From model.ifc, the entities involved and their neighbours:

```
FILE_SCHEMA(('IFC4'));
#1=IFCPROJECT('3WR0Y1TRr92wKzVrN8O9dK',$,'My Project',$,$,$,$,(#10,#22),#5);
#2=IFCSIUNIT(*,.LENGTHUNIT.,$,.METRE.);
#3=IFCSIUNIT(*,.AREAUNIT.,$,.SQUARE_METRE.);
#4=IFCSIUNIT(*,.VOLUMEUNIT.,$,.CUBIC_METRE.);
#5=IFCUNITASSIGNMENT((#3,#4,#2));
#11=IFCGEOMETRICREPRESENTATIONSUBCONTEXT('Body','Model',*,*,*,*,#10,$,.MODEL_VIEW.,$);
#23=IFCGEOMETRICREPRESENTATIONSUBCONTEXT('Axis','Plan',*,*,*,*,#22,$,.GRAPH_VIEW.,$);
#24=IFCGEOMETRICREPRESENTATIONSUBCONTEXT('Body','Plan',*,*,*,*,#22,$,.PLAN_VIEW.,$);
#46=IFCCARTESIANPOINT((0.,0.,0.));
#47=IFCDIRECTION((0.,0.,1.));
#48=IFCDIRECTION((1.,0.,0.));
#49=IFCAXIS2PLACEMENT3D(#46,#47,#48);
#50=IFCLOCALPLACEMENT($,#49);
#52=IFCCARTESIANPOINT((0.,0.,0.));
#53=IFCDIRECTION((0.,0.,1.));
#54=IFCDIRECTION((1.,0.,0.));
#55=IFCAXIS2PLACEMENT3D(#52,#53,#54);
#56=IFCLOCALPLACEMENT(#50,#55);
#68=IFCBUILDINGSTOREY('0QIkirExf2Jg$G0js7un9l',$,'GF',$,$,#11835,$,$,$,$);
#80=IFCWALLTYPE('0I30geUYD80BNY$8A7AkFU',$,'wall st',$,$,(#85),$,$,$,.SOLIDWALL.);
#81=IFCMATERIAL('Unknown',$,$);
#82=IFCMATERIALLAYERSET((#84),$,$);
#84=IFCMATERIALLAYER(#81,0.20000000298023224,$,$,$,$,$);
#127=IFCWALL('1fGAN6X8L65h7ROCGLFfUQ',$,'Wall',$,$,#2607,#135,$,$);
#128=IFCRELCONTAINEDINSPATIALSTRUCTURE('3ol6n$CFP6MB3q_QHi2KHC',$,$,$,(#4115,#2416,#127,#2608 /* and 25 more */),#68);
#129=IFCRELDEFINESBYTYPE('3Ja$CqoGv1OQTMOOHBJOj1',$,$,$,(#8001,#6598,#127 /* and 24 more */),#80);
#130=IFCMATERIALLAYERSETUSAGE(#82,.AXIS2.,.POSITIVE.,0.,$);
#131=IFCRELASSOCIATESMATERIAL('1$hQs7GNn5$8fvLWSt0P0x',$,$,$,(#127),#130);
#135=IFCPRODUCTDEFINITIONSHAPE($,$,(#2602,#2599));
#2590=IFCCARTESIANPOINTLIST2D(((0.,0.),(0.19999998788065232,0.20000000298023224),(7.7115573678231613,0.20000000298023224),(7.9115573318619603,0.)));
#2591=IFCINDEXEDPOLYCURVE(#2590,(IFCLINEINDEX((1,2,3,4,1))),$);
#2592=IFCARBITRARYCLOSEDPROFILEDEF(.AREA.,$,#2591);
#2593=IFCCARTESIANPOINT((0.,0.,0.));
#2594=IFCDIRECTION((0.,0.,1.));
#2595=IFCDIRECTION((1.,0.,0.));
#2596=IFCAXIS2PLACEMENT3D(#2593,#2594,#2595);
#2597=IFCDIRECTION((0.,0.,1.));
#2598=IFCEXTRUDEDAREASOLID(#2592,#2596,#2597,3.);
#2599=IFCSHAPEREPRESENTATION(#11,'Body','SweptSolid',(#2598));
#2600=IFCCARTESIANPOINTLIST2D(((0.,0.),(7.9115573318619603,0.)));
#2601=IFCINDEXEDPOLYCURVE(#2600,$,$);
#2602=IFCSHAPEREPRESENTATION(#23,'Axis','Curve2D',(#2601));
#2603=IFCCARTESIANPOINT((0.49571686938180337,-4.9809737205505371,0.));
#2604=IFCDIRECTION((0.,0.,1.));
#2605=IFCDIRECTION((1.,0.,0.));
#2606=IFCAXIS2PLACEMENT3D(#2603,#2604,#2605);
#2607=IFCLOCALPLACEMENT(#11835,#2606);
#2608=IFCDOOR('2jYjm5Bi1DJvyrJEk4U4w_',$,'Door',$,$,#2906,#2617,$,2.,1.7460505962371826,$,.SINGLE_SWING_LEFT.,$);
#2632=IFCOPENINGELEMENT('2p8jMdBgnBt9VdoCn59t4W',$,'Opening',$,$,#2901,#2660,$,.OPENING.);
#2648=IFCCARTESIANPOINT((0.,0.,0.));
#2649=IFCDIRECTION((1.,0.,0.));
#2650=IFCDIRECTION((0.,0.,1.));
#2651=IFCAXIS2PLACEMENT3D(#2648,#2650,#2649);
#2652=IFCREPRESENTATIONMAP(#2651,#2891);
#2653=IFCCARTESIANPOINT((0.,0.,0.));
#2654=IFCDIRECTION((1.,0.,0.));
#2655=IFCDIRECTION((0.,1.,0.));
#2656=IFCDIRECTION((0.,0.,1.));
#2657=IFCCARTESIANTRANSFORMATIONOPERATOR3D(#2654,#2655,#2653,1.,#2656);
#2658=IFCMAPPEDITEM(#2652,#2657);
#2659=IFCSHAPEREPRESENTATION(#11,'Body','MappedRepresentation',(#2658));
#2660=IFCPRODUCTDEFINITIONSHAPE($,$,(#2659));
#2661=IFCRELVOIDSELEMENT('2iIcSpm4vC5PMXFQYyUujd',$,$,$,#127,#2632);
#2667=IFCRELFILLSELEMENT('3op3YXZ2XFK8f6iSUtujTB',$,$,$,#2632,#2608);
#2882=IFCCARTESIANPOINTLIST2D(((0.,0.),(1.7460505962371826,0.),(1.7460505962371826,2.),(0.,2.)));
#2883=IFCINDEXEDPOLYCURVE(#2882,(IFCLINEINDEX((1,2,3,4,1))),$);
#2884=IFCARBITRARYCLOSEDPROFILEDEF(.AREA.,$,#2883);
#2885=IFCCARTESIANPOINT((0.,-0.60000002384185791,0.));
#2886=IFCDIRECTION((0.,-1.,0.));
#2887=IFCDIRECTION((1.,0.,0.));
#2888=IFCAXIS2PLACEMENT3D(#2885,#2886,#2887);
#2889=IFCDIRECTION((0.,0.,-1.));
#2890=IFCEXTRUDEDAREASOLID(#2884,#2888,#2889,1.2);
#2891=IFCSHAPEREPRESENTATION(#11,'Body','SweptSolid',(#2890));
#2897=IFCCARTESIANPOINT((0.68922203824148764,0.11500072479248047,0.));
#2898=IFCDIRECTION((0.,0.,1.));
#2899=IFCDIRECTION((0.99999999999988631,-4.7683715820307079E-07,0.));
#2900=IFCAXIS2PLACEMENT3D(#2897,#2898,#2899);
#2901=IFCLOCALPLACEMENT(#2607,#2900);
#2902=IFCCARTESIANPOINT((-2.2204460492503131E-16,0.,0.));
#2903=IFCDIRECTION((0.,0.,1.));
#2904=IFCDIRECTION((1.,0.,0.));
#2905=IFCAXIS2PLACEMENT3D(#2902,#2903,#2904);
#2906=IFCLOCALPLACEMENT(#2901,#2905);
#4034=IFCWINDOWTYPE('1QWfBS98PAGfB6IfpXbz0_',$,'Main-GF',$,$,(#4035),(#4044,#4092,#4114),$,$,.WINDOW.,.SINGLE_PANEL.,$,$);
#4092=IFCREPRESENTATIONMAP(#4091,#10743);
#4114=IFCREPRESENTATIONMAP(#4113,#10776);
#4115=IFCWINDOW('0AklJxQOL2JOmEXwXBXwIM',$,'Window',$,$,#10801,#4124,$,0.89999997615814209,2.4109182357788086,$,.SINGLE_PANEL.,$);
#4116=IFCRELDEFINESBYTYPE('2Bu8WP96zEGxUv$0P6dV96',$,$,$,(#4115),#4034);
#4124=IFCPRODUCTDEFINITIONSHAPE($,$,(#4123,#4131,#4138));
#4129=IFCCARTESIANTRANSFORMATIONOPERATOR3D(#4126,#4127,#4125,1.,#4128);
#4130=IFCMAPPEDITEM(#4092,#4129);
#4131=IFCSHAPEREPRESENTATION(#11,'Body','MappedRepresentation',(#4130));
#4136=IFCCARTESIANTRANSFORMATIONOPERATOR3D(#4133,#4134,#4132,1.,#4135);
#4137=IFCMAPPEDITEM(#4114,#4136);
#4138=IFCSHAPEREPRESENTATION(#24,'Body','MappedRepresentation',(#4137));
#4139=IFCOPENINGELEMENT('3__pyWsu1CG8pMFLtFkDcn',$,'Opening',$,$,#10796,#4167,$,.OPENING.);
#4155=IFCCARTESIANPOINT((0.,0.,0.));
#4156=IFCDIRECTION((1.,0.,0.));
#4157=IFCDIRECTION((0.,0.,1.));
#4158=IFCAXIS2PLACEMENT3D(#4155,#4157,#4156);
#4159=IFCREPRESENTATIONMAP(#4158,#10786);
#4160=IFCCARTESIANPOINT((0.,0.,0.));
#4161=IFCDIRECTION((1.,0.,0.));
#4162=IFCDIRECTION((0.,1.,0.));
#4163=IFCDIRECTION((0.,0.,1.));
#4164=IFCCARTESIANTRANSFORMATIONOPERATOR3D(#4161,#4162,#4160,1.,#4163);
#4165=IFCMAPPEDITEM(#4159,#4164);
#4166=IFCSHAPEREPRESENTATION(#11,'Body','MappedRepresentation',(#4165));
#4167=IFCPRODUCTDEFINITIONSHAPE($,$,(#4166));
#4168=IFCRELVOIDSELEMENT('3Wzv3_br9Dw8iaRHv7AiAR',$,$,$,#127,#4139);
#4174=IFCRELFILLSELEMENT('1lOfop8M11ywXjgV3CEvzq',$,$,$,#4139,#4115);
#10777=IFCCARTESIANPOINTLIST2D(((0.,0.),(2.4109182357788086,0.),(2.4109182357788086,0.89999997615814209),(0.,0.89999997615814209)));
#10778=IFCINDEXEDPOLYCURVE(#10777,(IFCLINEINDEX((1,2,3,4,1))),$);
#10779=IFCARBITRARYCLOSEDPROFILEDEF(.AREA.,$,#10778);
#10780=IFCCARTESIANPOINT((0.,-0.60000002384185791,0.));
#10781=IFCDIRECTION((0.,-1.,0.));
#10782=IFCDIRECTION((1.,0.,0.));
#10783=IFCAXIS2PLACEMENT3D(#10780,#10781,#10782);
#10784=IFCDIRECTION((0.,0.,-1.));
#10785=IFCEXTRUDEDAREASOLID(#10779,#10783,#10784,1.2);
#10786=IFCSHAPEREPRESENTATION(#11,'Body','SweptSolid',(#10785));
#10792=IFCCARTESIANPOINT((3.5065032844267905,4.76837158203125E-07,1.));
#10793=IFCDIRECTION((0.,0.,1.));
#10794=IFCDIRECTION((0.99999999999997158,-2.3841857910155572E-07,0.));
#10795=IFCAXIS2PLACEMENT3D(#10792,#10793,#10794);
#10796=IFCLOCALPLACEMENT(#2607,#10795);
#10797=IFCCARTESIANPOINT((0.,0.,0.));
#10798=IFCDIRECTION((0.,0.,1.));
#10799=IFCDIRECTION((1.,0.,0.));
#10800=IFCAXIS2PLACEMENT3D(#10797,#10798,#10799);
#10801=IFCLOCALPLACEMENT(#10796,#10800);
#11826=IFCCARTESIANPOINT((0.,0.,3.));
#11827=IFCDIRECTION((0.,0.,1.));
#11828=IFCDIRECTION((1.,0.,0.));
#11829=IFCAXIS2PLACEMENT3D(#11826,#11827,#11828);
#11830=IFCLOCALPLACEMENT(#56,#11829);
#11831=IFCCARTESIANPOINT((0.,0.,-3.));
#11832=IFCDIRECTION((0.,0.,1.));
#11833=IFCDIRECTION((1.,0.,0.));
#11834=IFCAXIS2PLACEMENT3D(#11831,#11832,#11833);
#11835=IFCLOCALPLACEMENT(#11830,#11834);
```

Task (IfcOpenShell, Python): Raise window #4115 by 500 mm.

```python
import numpy as np
import ifcopenshell
import ifcopenshell.api.geometry
import ifcopenshell.util.placement
import ifcopenshell.util.unit

model = ifcopenshell.open("model.ifc")
unit_scale = ifcopenshell.util.unit.calculate_unit_scale(model)

window = model.by_guid("0AklJxQOL2JOmEXwXBXwIM")
opening = window.FillsVoids[0].RelatingOpeningElement
dz = 0.5 / unit_scale

shift = np.array([0.0, 0.0, dz])
# The window is placed relative to its opening, so it follows when the opening moves.
matrix = ifcopenshell.util.placement.get_local_placement(opening.ObjectPlacement)
matrix[:3, 3] += shift
ifcopenshell.api.geometry.edit_object_placement(
    model, product=opening, matrix=matrix, is_si=False, should_transform_children=True
)

print(f"moved by {dz * unit_scale:+.3f} m")

model.write("model-out.ifc")
```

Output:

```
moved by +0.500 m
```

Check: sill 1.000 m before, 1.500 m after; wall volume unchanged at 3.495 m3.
